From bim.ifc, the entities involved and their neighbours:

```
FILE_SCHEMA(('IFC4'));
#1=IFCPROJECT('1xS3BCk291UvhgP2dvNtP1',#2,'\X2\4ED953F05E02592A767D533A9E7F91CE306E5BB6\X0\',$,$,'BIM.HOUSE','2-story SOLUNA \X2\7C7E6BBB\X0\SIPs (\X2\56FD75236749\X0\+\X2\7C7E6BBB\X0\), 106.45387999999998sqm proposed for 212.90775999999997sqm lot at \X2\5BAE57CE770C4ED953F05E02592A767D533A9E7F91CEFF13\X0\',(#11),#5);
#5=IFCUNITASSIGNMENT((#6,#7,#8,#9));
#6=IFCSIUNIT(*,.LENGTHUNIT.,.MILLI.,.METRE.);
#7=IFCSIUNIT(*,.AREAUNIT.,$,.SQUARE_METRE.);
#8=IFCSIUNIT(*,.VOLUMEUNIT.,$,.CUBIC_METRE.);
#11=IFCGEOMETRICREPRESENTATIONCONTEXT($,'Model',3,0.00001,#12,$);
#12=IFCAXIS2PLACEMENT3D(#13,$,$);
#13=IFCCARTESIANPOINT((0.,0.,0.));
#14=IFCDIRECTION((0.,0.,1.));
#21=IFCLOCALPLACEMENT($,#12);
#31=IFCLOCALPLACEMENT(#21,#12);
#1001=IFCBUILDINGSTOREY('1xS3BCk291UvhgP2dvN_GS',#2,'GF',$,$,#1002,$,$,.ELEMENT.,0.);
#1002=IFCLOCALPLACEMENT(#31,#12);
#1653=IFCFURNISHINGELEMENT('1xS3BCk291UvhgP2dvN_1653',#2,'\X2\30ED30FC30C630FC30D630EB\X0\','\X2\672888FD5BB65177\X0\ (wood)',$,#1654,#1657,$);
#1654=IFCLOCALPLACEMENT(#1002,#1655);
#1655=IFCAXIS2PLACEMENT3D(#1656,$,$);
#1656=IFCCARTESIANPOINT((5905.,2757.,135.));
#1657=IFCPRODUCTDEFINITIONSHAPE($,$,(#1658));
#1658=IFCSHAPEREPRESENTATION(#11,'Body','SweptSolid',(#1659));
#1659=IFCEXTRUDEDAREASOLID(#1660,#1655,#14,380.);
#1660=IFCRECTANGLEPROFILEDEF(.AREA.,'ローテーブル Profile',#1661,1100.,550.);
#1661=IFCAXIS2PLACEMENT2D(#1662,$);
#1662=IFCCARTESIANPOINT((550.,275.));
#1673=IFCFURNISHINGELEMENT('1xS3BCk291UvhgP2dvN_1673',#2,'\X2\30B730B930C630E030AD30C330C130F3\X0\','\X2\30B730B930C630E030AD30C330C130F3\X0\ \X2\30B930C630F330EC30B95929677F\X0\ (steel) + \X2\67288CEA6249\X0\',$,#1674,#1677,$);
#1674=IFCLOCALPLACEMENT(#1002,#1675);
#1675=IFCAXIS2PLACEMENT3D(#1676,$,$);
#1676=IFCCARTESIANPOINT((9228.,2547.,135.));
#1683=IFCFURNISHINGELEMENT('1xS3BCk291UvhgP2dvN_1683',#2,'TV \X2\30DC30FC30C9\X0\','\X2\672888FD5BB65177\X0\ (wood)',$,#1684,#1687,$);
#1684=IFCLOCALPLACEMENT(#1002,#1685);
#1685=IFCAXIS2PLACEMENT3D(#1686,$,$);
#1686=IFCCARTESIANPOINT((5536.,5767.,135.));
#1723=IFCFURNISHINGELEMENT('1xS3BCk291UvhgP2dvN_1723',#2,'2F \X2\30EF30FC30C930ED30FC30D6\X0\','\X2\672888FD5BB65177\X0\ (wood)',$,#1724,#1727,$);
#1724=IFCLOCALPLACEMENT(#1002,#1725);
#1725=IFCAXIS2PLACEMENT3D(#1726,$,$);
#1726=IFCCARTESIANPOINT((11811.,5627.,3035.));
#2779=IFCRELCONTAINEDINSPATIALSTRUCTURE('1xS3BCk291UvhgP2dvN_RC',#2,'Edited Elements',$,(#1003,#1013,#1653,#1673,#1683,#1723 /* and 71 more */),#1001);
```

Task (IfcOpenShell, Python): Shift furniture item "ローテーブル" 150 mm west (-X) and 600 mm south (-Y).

```python
import ifcopenshell
import ifcopenshell.api.geometry
import ifcopenshell.util.placement

model = ifcopenshell.open("bim.ifc")

item = model.by_guid("1xS3BCk291UvhgP2dvN_1653")
matrix = ifcopenshell.util.placement.get_local_placement(item.ObjectPlacement)
matrix[0, 3] -= 150.0
matrix[1, 3] -= 600.0
ifcopenshell.api.geometry.edit_object_placement(model, product=item, matrix=matrix, is_si=False)

print(ifcopenshell.util.placement.get_local_placement(item.ObjectPlacement).round(3) + 0.0)

model.write("bim_updated.ifc")
```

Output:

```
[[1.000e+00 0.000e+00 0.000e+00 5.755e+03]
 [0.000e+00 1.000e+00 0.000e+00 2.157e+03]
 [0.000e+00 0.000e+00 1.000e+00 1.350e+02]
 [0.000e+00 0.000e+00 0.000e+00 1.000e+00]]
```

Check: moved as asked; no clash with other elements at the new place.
